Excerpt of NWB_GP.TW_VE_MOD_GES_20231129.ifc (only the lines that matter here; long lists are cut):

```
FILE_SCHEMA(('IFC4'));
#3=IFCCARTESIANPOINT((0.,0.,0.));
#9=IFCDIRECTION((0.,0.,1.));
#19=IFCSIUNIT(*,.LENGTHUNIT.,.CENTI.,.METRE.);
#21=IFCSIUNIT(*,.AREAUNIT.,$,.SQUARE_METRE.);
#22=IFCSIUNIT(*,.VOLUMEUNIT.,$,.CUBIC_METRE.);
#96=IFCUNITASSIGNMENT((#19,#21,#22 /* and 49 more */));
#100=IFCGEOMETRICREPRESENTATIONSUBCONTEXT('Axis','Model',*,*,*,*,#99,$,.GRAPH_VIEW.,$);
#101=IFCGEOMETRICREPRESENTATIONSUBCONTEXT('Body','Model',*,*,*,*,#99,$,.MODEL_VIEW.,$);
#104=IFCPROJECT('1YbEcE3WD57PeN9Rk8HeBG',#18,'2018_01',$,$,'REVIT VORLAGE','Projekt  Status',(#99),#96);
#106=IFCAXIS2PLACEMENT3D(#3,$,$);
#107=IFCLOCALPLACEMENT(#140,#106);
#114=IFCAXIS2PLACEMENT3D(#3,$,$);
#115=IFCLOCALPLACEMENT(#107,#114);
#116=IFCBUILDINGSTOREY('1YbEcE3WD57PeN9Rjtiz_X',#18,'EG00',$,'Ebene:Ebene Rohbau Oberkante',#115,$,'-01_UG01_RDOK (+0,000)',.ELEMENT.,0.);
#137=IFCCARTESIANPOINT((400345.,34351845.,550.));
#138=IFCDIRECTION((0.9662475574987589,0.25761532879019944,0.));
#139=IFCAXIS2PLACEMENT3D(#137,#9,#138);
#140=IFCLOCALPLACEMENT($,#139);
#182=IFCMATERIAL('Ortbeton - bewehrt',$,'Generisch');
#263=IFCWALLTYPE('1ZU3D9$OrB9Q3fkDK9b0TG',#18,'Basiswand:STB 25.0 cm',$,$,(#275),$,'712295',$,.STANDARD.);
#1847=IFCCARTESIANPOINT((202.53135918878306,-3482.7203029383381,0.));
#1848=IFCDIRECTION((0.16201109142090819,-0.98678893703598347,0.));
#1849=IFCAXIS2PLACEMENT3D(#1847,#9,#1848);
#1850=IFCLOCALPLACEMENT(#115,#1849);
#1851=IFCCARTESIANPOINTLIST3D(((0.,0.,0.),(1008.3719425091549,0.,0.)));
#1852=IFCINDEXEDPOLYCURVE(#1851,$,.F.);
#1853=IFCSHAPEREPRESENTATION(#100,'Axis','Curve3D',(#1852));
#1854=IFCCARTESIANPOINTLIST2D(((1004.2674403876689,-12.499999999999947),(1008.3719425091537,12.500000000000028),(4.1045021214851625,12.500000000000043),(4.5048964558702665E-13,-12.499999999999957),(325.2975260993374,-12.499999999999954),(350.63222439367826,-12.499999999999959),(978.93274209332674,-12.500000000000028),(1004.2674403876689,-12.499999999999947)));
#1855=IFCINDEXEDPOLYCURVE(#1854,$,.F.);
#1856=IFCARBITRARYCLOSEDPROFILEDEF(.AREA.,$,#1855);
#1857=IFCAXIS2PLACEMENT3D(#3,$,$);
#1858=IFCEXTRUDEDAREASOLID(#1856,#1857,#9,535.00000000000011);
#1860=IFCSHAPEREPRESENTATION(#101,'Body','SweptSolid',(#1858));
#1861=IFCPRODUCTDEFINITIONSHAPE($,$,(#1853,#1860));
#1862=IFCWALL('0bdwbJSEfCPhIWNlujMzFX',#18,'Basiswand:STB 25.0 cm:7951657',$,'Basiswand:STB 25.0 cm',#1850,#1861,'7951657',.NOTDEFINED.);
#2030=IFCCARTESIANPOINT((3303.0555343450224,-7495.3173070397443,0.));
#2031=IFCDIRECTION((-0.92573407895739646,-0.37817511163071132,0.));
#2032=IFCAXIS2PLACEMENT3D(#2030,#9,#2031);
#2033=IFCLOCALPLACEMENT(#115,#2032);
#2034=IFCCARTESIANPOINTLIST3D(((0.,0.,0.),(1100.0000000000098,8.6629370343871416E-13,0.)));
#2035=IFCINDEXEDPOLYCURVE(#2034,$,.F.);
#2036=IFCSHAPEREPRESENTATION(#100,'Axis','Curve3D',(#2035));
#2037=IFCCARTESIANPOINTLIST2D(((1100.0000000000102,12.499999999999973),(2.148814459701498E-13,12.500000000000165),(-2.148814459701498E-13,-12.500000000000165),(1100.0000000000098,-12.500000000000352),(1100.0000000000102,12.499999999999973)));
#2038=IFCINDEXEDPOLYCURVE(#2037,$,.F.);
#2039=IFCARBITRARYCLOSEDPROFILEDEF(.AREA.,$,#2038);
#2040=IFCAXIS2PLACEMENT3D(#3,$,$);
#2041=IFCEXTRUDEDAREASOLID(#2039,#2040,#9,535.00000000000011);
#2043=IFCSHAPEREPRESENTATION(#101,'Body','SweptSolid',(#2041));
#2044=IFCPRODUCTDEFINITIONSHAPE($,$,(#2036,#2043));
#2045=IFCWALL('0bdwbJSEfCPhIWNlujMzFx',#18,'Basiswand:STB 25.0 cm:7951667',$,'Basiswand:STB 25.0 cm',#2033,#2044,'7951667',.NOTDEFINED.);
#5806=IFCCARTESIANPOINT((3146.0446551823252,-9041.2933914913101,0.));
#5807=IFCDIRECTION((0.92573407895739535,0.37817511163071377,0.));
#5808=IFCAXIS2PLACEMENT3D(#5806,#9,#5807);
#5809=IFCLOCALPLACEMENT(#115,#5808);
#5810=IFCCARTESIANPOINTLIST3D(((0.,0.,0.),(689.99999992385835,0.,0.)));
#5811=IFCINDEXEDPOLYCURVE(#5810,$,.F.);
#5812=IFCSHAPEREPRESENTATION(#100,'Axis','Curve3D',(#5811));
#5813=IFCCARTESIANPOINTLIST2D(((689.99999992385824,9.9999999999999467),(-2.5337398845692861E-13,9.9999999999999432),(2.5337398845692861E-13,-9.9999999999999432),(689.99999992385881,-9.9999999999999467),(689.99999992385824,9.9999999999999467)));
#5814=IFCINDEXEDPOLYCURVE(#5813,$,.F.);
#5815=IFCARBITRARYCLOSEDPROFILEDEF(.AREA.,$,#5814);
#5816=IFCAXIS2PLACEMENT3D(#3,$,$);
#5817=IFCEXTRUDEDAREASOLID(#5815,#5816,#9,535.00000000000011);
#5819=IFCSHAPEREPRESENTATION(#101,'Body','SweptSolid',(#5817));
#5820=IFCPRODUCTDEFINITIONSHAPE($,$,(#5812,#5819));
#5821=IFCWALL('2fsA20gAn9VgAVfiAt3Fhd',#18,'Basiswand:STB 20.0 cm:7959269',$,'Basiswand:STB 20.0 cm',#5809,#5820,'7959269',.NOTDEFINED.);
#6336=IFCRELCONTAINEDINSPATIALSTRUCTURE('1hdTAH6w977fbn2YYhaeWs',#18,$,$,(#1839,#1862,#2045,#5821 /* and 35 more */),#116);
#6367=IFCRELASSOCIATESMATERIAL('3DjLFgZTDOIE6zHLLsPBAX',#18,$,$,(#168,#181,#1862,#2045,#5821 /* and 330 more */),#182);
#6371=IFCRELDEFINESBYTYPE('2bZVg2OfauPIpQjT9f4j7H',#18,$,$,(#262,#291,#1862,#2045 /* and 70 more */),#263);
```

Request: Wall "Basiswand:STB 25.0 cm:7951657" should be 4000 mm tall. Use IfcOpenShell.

```python
import ifcopenshell
import ifcopenshell.geom
import ifcopenshell.util.representation
import ifcopenshell.util.shape
import ifcopenshell.util.unit

model = ifcopenshell.open("NWB_GP.TW_VE_MOD_GES_20231129.ifc")
unit_scale = ifcopenshell.util.unit.calculate_unit_scale(model)
settings = ifcopenshell.geom.settings()


def volume(element):
    """Net volume in cubic metres, openings subtracted."""
    shape = ifcopenshell.geom.create_shape(settings, element)
    return ifcopenshell.util.shape.get_volume(shape.geometry)


wall = model.by_guid("0bdwbJSEfCPhIWNlujMzFX")
before = volume(wall)

body = ifcopenshell.util.representation.get_representation(wall, "Model", "Body")
solid = body.Items[0]
old_height = solid.Depth
solid.Depth = 4 / unit_scale
after = volume(wall)

print(f"height {old_height:g} -> {solid.Depth:g}, volume {before:.3f} -> {after:.3f} m3")

model.write("NWB_GP.TW_VE_MOD_GES_20231129_updated.ifc")
```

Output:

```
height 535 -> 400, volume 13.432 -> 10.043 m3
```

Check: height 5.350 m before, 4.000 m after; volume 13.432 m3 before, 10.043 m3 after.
